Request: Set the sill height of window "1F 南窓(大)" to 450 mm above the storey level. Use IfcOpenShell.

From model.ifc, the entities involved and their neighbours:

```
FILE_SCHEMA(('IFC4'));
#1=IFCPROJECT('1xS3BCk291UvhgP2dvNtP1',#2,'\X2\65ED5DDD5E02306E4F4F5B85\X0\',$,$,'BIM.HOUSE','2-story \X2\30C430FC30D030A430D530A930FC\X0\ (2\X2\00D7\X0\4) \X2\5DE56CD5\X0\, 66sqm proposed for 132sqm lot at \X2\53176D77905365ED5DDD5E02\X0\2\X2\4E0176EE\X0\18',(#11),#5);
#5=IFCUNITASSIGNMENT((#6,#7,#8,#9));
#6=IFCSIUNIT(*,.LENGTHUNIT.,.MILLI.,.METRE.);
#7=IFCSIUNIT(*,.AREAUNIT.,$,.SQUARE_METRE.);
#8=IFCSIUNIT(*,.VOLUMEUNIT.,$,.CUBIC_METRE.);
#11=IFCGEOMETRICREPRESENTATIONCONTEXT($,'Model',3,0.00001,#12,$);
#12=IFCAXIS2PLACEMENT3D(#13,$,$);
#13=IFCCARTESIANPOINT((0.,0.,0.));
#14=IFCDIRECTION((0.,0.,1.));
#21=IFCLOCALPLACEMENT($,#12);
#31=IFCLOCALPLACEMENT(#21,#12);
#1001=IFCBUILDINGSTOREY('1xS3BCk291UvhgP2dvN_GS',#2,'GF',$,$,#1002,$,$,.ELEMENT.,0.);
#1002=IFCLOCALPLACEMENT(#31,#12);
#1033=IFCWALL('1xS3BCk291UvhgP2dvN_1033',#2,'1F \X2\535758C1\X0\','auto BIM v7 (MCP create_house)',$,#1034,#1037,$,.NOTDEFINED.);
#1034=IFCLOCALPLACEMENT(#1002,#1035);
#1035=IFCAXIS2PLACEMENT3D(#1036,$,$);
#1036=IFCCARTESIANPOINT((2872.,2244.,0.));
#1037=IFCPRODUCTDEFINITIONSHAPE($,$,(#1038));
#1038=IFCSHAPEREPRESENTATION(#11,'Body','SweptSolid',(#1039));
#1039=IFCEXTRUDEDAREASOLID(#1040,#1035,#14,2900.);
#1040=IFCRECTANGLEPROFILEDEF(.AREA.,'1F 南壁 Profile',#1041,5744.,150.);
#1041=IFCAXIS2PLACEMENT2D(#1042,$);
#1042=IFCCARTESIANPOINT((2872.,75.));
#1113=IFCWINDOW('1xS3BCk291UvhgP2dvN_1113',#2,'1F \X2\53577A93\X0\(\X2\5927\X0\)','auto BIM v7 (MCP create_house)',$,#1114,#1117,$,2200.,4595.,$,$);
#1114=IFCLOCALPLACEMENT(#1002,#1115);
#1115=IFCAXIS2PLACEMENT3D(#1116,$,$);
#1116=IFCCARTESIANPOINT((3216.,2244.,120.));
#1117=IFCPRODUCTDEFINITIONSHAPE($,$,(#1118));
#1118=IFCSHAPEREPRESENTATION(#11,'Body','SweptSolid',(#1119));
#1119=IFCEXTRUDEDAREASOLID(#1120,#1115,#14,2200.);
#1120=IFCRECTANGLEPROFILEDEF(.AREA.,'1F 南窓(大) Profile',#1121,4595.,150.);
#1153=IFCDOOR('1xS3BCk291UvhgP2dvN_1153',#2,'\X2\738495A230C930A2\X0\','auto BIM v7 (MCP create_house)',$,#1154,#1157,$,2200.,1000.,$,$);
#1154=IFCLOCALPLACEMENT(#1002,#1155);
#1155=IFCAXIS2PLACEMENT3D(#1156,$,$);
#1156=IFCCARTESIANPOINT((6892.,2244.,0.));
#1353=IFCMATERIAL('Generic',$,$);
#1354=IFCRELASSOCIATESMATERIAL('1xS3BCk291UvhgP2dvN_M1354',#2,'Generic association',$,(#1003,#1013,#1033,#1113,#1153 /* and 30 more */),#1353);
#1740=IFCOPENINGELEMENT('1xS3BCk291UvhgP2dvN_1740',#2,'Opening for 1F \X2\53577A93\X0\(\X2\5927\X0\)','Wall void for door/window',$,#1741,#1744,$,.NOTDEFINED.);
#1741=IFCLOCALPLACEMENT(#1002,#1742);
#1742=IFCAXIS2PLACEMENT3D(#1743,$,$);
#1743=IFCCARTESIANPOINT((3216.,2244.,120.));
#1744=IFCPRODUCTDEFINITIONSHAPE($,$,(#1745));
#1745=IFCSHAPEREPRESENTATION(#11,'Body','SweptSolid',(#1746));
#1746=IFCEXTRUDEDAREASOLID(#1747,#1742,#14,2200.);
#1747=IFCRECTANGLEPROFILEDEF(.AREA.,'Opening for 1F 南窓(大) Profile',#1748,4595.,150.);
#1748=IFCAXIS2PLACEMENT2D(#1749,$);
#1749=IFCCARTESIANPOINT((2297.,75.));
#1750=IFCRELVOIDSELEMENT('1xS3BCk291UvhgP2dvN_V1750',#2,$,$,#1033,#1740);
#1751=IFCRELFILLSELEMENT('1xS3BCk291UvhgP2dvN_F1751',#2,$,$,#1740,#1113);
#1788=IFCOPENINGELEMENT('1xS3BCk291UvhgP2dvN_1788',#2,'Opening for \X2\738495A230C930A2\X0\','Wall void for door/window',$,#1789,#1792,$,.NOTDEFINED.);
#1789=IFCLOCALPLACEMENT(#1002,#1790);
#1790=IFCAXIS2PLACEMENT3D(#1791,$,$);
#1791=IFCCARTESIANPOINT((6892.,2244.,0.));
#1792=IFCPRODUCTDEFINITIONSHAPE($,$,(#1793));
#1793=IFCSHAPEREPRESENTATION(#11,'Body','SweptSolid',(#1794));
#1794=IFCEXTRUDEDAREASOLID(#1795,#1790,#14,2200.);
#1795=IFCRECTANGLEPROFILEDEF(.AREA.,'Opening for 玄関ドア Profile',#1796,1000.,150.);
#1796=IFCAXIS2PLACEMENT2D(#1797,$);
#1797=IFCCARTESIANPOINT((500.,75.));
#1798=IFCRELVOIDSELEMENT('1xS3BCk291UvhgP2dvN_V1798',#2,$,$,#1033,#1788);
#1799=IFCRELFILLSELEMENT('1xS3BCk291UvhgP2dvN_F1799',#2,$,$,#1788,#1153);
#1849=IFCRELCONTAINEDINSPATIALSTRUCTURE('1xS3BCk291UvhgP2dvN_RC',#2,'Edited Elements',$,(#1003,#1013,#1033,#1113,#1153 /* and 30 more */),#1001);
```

```python
import numpy as np
import ifcopenshell
import ifcopenshell.api.geometry
import ifcopenshell.geom
import ifcopenshell.util.element
import ifcopenshell.util.placement
import ifcopenshell.util.shape
import ifcopenshell.util.unit

model = ifcopenshell.open("model.ifc")
unit_scale = ifcopenshell.util.unit.calculate_unit_scale(model)

window = model.by_guid("1xS3BCk291UvhgP2dvN_1113")
opening = window.FillsVoids[0].RelatingOpeningElement
storey = ifcopenshell.util.element.get_container(window, ifc_class="IfcBuildingStorey")
level = ifcopenshell.util.placement.get_local_placement(storey.ObjectPlacement)[2, 3]

# The opening's origin need not be at the sill, so measure its lowest point.
shape = ifcopenshell.geom.create_shape(ifcopenshell.geom.settings(), opening)
bottom = ifcopenshell.util.shape.get_shape_bottom_elevation(shape, shape.geometry) / unit_scale
dz = level + 450.0 - bottom

shift = np.array([0.0, 0.0, dz])
# The window is not placed relative to its opening, so move both.
for product in (opening, window):
    matrix = ifcopenshell.util.placement.get_local_placement(product.ObjectPlacement)
    matrix[:3, 3] += shift
    ifcopenshell.api.geometry.edit_object_placement(model, product=product, matrix=matrix, is_si=False)

print(f"moved by {dz * unit_scale:+.3f} m")

model.write("model_edited.ifc")
```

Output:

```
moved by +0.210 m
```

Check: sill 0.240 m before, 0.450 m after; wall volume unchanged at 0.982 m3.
